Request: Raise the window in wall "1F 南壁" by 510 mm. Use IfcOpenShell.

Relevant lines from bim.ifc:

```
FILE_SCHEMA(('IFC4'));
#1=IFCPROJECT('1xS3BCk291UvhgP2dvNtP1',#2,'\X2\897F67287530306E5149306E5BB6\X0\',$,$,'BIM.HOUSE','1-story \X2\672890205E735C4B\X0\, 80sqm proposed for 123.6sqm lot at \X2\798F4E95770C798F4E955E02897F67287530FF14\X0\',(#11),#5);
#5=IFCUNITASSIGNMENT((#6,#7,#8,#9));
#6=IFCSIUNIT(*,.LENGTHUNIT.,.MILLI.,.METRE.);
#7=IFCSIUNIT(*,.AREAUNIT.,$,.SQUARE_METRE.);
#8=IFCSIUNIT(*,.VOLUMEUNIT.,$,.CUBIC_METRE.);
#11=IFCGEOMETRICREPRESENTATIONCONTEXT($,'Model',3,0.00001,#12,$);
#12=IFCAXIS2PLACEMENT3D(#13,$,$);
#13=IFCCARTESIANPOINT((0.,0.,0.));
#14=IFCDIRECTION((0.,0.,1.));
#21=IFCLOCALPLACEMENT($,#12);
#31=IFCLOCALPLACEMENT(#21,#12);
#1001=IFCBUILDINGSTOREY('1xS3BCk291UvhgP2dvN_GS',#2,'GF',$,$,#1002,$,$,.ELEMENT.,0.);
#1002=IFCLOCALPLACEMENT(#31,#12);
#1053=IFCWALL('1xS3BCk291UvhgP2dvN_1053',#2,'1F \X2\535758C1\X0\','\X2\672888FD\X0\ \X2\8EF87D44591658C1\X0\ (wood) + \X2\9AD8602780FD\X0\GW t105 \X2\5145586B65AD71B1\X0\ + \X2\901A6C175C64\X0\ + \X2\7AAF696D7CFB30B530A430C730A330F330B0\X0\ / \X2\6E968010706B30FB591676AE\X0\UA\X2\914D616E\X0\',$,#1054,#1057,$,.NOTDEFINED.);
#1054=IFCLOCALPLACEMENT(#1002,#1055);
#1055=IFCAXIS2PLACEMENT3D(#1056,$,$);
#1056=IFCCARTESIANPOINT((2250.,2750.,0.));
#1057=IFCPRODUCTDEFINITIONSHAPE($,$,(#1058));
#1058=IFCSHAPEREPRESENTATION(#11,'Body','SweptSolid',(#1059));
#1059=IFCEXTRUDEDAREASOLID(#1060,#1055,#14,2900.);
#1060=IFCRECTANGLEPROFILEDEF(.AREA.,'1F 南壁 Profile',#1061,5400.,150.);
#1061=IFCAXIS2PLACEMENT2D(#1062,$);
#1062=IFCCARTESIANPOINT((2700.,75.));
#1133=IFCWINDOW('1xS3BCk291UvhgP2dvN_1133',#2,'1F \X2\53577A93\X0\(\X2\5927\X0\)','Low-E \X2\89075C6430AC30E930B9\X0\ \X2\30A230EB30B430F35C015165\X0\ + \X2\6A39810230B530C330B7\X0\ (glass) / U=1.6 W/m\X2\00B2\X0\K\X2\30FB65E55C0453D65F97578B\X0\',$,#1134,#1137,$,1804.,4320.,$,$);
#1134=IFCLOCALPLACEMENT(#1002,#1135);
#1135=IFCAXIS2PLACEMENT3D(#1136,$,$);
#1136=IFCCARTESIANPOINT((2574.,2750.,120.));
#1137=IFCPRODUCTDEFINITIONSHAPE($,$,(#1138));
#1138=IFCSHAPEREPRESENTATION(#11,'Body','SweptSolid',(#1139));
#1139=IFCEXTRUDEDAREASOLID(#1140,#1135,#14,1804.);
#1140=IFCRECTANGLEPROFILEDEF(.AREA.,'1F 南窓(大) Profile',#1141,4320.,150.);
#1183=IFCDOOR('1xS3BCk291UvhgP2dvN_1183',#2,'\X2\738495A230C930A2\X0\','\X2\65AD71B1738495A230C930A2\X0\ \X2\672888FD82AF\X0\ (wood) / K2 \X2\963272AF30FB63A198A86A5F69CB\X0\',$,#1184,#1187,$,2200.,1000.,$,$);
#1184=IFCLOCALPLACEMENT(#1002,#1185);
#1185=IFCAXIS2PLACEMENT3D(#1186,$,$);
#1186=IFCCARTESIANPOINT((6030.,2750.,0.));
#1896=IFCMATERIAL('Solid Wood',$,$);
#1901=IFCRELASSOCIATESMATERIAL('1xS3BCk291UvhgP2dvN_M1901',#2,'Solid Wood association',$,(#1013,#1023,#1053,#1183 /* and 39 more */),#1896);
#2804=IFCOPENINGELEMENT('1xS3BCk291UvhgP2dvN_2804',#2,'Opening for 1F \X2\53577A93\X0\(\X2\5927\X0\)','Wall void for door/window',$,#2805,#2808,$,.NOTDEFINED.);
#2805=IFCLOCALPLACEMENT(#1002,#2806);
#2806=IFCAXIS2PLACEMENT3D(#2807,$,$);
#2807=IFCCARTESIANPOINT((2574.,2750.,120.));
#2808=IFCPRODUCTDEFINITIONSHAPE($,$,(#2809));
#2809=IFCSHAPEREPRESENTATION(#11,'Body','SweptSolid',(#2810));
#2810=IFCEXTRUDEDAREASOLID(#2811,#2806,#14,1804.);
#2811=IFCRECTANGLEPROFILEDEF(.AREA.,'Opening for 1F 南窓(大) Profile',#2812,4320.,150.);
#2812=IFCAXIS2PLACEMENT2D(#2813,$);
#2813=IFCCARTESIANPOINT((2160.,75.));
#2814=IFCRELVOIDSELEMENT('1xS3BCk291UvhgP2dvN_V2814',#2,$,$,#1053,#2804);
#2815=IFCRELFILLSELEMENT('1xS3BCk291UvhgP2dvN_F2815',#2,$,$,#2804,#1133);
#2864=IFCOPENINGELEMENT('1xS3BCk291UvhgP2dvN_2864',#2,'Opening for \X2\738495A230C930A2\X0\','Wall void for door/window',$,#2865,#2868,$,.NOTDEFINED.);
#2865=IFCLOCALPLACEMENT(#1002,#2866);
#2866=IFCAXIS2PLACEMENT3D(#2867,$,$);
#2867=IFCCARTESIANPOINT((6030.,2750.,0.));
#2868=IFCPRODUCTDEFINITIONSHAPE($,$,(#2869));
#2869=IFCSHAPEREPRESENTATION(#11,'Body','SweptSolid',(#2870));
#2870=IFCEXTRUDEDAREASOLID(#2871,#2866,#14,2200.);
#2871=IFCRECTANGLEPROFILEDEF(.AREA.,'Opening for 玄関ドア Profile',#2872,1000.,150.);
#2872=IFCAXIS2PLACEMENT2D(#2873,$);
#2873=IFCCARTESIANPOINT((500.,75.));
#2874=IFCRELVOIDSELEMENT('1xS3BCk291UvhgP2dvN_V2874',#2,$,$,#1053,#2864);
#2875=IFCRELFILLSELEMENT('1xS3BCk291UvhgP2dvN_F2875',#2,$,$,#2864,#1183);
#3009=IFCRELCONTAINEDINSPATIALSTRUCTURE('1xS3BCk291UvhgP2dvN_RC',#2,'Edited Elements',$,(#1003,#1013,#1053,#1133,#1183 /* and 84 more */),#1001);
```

```python
import numpy as np
import ifcopenshell
import ifcopenshell.api.geometry
import ifcopenshell.util.placement
import ifcopenshell.util.unit

model = ifcopenshell.open("bim.ifc")
unit_scale = ifcopenshell.util.unit.calculate_unit_scale(model)

window = model.by_guid("1xS3BCk291UvhgP2dvN_1133")
opening = window.FillsVoids[0].RelatingOpeningElement
dz = 510.0

shift = np.array([0.0, 0.0, dz])
# The window is not placed relative to its opening, so move both.
for product in (opening, window):
    matrix = ifcopenshell.util.placement.get_local_placement(product.ObjectPlacement)
    matrix[:3, 3] += shift
    ifcopenshell.api.geometry.edit_object_placement(model, product=product, matrix=matrix, is_si=False)

print(f"moved by {dz * unit_scale:+.3f} m")

model.write("bim-out.ifc")
```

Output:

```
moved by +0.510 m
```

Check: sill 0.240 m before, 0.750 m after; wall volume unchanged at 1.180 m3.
